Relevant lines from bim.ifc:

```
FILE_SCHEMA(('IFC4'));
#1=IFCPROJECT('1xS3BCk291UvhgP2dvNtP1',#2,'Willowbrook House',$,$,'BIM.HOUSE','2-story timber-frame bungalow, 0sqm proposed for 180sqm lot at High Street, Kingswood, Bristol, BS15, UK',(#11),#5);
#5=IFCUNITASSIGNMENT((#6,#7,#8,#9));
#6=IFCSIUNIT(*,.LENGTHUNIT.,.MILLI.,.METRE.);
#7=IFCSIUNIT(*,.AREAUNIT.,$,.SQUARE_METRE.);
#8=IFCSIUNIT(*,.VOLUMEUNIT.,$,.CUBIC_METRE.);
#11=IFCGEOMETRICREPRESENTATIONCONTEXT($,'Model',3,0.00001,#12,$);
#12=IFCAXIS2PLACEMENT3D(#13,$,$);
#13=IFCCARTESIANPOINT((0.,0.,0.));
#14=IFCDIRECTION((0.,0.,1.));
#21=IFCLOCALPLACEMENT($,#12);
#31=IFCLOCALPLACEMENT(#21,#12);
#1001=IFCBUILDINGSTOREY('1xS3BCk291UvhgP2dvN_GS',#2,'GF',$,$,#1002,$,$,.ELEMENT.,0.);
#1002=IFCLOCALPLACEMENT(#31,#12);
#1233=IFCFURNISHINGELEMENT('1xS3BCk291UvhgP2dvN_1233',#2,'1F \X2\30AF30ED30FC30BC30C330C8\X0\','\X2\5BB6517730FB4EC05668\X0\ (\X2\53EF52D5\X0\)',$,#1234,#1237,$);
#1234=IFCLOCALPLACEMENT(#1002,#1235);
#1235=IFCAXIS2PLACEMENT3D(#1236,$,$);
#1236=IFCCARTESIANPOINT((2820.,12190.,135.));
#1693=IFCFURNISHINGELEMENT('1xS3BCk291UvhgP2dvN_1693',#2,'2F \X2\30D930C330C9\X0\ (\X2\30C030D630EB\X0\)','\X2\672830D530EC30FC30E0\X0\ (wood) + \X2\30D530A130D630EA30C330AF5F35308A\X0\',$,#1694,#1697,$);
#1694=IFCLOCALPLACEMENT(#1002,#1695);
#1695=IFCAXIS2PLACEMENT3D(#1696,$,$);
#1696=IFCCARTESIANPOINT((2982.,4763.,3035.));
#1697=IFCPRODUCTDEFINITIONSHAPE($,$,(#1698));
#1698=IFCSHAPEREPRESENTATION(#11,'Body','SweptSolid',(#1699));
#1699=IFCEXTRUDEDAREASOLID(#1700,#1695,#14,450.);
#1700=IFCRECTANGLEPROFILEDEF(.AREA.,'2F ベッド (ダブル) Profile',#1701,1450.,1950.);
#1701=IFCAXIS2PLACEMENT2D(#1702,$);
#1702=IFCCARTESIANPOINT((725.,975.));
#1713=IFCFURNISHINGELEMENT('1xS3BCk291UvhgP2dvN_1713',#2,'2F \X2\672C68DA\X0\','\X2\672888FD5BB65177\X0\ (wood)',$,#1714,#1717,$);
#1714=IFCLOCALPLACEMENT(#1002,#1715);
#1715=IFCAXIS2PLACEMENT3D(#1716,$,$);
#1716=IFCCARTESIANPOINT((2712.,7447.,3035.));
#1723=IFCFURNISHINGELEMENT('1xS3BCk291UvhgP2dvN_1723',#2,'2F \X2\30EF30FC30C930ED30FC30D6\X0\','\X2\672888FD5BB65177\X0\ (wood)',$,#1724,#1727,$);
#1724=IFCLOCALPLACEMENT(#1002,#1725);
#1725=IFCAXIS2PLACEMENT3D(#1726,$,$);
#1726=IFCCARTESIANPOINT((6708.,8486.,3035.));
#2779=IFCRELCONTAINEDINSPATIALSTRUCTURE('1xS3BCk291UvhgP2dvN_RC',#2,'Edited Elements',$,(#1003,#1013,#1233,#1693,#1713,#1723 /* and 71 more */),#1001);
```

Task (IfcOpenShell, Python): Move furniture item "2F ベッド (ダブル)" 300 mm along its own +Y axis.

```python
import ifcopenshell
import ifcopenshell.api.geometry
import ifcopenshell.util.placement
import ifcopenshell.util.unit

model = ifcopenshell.open("bim.ifc")
unit_scale = ifcopenshell.util.unit.calculate_unit_scale(model)

item = model.by_guid("1xS3BCk291UvhgP2dvN_1693")
matrix = ifcopenshell.util.placement.get_local_placement(item.ObjectPlacement)
matrix[:3, 3] += matrix[:3, 1] * 0.3 / unit_scale
ifcopenshell.api.geometry.edit_object_placement(model, product=item, matrix=matrix, is_si=False)

print(ifcopenshell.util.placement.get_local_placement(item.ObjectPlacement).round(3) + 0.0)

model.write("bim_edited.ifc")
```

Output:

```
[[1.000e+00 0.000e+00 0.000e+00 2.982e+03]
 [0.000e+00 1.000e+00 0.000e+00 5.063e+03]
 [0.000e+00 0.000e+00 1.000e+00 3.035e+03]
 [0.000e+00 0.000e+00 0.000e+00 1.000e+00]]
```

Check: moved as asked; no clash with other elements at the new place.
